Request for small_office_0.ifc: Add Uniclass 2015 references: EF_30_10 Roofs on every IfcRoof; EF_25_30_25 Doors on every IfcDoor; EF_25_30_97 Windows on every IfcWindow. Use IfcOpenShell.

First a look at what the model holds.

```python
import ifcopenshell

model = ifcopenshell.open("small_office_0.ifc")
print(model.schema)
print("classifications:", [c.Name for c in model.by_type("IfcClassification")])
for ifc_class in ("IfcDoor", "IfcRoof", "IfcStair", "IfcWall", "IfcWindow"):
    print(ifc_class, len(model.by_type(ifc_class)))
```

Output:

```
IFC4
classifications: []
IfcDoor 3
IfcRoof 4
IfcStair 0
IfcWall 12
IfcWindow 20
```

```python
import ifcopenshell
import ifcopenshell.api.classification

model = ifcopenshell.open("small_office_0.ifc")

system = ifcopenshell.api.classification.add_classification(model, classification="Uniclass 2015")

codes = {
    "IfcRoof": ("EF_30_10", "Roofs"),
    "IfcDoor": ("EF_25_30_25", "Doors"),
    "IfcWindow": ("EF_25_30_97", "Windows"),
}
for ifc_class, (code, name) in codes.items():
    products = model.by_type(ifc_class)
    ifcopenshell.api.classification.add_reference(
        model, products=products, classification=system, identification=code, name=name
    )
    print(code, len(products))

model.write("small_office_0_updated.ifc")
```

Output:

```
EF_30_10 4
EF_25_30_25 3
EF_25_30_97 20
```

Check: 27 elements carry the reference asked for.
